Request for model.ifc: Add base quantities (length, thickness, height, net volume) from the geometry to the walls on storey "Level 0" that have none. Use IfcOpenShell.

First a look at what the model holds.

```python
import ifcopenshell
import ifcopenshell.util.element
import ifcopenshell.util.unit

model = ifcopenshell.open("model.ifc")
print(model.schema)
for unit_type in ("LENGTHUNIT", "AREAUNIT", "VOLUMEUNIT"):
    print(unit_type, ifcopenshell.util.unit.calculate_unit_scale(model, unit_type))
storey = next(s for s in model.by_type("IfcBuildingStorey") if s.Name == "Level 0")
walls = [e for e in ifcopenshell.util.element.get_decomposition(storey) if e.is_a("IfcWall")]
for e in sorted(walls, key=lambda e: e.id()):
    print(e.id(), e.is_a(), e.Name, list(ifcopenshell.util.element.get_psets(e, qtos_only=True)), sep=" | ")
```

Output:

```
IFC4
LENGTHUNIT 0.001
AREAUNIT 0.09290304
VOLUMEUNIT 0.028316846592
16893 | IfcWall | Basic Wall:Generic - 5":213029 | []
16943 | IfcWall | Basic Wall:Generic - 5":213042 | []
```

```python
import ifcopenshell
import ifcopenshell.api.pset
import ifcopenshell.geom
import ifcopenshell.util.element
import ifcopenshell.util.shape
import ifcopenshell.util.unit

model = ifcopenshell.open("model.ifc")
unit_scale = ifcopenshell.util.unit.calculate_unit_scale(model)
volume_scale = ifcopenshell.util.unit.calculate_unit_scale(model, "VOLUMEUNIT")
settings = ifcopenshell.geom.settings()

storey = next(s for s in model.by_type("IfcBuildingStorey") if s.Name == "Level 0")
walls = [e for e in ifcopenshell.util.element.get_decomposition(storey) if e.is_a("IfcWall")]

for e in sorted(walls, key=lambda e: e.id()):
    if ifcopenshell.util.element.get_psets(e, qtos_only=True, should_inherit=False):
        continue
    # Geometry comes back in metres, in the element's own axes.
    shape = ifcopenshell.geom.create_shape(settings, e)
    values = {
        "Length": ifcopenshell.util.shape.get_x(shape.geometry) / unit_scale,
        "Width": ifcopenshell.util.shape.get_y(shape.geometry) / unit_scale,
        "Height": ifcopenshell.util.shape.get_z(shape.geometry) / unit_scale,
        "NetVolume": ifcopenshell.util.shape.get_volume(shape.geometry) / volume_scale,
    }
    qto = ifcopenshell.api.pset.add_qto(model, product=e, name="Qto_WallBaseQuantities")
    ifcopenshell.api.pset.edit_qto(model, qto=qto, properties=values)
    print(e.id(), {k: round(v, 3) for k, v in values.items()})

model.write("model-out.ifc")
```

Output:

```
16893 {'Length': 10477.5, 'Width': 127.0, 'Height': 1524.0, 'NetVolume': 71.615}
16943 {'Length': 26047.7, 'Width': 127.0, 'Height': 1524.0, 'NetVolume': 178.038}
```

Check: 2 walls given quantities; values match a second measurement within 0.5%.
